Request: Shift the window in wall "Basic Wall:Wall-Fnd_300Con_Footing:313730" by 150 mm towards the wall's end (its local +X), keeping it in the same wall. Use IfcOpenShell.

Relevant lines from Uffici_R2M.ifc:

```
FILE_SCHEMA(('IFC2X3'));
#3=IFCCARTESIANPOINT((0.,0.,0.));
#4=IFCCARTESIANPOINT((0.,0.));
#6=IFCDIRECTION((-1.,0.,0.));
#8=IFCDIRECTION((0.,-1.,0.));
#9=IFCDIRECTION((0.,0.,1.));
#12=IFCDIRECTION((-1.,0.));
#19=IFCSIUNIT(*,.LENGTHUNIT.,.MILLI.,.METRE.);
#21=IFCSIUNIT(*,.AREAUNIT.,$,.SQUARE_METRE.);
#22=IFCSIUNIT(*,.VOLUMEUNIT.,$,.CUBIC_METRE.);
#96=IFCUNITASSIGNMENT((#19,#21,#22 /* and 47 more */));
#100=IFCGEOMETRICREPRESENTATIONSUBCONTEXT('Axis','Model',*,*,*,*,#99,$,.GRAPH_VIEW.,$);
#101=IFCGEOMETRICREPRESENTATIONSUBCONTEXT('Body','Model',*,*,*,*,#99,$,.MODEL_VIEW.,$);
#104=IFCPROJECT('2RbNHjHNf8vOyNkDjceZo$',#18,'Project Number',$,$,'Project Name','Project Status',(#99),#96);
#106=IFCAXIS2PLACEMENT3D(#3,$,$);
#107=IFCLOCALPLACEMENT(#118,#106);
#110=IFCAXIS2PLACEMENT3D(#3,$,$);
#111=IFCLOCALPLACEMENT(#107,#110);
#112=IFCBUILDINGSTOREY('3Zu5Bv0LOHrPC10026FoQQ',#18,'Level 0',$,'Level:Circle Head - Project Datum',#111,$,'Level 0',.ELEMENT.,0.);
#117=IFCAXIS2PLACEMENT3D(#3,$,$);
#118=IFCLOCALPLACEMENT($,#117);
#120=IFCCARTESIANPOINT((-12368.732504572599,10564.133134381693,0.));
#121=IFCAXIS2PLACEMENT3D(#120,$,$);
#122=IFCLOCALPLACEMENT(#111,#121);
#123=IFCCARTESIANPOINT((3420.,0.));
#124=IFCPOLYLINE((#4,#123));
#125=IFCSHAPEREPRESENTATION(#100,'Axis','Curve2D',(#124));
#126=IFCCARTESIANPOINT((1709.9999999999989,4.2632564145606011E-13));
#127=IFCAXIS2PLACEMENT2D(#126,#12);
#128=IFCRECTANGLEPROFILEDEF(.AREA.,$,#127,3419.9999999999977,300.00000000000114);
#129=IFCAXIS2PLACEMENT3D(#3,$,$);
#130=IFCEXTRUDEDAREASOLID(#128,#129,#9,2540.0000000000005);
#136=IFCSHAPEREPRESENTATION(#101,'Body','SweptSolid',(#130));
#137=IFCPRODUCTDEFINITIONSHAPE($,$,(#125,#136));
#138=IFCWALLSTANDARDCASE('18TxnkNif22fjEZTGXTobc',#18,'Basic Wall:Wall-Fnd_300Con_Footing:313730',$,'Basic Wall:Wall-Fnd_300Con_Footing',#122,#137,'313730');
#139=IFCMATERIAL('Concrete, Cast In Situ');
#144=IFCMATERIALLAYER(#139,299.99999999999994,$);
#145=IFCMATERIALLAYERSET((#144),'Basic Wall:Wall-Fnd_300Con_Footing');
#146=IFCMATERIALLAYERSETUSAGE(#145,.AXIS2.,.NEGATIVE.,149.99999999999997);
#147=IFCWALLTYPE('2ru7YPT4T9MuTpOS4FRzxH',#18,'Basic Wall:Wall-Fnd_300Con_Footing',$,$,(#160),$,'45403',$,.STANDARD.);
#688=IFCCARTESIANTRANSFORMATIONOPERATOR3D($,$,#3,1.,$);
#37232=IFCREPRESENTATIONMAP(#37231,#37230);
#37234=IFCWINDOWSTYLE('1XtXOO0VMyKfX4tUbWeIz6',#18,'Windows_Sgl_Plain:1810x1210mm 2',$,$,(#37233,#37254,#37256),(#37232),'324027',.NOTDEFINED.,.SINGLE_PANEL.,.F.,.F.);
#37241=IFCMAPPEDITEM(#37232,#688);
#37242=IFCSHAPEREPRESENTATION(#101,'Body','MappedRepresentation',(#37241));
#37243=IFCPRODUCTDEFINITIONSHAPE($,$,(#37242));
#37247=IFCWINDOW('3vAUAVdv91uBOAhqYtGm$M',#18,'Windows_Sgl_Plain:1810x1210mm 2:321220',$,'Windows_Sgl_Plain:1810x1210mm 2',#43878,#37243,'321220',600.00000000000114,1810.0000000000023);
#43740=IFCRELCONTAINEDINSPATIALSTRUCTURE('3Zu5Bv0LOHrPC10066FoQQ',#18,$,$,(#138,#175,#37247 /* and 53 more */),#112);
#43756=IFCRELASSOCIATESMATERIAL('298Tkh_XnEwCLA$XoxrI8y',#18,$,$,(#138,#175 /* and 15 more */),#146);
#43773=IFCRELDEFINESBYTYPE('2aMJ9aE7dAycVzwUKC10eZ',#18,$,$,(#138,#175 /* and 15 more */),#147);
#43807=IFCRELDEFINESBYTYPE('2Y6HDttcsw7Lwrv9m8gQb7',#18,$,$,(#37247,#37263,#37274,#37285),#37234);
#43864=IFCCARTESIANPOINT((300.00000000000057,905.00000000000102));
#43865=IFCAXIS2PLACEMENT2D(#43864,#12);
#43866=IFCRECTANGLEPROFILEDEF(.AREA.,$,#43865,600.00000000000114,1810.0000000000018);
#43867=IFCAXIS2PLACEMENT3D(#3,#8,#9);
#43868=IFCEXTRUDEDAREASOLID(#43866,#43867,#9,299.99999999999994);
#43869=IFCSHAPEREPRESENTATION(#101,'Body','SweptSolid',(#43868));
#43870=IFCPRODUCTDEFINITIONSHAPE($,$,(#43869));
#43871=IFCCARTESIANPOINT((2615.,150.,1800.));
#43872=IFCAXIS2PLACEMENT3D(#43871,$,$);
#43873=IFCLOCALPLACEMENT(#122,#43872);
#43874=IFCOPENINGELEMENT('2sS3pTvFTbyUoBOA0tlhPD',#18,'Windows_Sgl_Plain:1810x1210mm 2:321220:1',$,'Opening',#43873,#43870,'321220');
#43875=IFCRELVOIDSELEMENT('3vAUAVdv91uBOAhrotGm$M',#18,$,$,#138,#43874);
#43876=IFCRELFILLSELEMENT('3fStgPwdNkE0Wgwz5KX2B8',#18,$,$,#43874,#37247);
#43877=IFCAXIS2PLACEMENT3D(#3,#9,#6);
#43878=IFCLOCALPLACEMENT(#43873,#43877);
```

```python
import ifcopenshell
import ifcopenshell.api.geometry
import ifcopenshell.util.placement

model = ifcopenshell.open("Uffici_R2M.ifc")

window = model.by_id(37247)
opening = window.FillsVoids[0].RelatingOpeningElement
wall = opening.VoidsElements[0].RelatingBuildingElement

wall_matrix = ifcopenshell.util.placement.get_local_placement(wall.ObjectPlacement)
shift = wall_matrix[:3, 0] * 150.0
before = ifcopenshell.util.placement.get_local_placement(window.ObjectPlacement)[:3, 3].copy()

# The window is placed relative to its opening, so it follows when the opening moves.
matrix = ifcopenshell.util.placement.get_local_placement(opening.ObjectPlacement)
matrix[:3, 3] += shift
ifcopenshell.api.geometry.edit_object_placement(
    model, product=opening, matrix=matrix, is_si=False, should_transform_children=True
)

after = ifcopenshell.util.placement.get_local_placement(window.ObjectPlacement)[:3, 3]
print("window moved by", (after - before).round(3) + 0.0)

model.write("Uffici_R2M_edited.ifc")
```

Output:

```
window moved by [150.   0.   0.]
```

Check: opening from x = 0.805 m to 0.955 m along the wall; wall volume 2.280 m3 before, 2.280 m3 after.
